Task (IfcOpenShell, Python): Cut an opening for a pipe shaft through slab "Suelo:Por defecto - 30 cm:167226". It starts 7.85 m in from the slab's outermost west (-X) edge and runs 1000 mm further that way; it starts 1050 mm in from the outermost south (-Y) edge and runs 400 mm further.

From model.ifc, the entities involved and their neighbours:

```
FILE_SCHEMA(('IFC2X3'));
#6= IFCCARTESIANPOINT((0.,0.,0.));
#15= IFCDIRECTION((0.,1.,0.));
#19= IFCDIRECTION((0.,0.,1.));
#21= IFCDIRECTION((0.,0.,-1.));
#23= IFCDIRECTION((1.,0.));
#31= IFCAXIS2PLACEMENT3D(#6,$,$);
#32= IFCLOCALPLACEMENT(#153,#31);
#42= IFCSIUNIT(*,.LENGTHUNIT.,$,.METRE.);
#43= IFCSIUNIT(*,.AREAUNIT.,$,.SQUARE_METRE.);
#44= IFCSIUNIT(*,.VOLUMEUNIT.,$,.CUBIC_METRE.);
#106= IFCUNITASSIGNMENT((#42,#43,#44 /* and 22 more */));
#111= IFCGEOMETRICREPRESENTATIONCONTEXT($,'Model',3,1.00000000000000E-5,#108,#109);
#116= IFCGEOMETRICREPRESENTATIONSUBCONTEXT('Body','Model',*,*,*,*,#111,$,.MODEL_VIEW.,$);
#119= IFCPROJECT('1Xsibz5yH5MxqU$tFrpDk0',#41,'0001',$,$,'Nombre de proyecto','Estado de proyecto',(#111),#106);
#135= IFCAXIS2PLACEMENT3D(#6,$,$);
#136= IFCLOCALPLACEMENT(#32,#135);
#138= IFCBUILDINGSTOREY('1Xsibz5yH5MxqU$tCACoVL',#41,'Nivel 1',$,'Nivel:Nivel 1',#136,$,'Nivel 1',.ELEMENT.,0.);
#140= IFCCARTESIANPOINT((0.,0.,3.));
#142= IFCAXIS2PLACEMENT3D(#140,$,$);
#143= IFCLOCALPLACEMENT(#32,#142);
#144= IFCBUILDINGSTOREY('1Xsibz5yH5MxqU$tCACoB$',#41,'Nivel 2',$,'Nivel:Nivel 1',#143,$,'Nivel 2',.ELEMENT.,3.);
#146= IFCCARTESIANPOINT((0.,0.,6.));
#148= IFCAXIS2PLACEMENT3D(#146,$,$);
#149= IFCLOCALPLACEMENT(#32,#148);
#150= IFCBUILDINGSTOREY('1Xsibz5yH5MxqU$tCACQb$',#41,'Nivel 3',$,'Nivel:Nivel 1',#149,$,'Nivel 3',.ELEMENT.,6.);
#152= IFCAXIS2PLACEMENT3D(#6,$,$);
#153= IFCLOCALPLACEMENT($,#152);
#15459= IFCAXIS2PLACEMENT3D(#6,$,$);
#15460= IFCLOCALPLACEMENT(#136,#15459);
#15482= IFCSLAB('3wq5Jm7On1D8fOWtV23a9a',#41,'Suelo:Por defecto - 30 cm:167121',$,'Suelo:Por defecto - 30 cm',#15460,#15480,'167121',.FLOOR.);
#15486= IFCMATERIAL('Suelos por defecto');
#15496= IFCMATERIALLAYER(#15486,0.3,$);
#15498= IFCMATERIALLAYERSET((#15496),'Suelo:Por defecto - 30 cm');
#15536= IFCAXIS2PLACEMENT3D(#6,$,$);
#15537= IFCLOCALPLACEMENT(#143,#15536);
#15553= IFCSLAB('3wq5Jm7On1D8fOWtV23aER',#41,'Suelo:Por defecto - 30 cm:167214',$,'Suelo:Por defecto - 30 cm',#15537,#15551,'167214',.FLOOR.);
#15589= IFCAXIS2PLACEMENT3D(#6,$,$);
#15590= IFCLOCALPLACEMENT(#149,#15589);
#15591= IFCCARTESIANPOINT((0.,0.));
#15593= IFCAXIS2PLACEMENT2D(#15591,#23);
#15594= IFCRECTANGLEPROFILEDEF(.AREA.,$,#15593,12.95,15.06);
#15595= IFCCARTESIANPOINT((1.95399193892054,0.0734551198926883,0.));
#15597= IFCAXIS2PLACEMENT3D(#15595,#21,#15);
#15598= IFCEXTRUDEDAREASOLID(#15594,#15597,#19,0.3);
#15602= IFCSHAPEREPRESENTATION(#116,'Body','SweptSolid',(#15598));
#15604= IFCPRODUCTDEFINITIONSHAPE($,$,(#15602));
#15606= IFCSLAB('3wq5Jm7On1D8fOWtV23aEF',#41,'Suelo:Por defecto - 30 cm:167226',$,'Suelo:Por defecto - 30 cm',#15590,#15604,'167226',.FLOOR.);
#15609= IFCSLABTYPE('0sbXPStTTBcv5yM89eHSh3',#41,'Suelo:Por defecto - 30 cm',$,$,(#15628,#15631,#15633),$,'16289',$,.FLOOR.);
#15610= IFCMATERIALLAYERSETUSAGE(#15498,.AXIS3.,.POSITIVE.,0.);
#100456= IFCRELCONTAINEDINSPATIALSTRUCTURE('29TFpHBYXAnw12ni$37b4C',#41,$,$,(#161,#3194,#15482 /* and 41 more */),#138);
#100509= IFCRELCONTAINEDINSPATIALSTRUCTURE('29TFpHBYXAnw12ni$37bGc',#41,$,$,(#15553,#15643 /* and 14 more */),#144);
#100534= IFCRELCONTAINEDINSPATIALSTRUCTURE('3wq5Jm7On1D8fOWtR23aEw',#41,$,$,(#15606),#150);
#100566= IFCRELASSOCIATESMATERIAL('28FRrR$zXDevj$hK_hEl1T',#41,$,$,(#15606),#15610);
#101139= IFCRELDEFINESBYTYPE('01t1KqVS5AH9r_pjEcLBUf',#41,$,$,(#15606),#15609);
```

```python
import numpy as np
import ifcopenshell
import ifcopenshell.api.feature
import ifcopenshell.api.geometry
import ifcopenshell.api.root
import ifcopenshell.geom
import ifcopenshell.util.placement
import ifcopenshell.util.representation
import ifcopenshell.util.shape
import ifcopenshell.util.unit

model = ifcopenshell.open("model.ifc")
unit_scale = ifcopenshell.util.unit.calculate_unit_scale(model)
settings = ifcopenshell.geom.settings()


def volume(element):
    """Net volume in cubic metres, openings subtracted."""
    shape = ifcopenshell.geom.create_shape(settings, element)
    return ifcopenshell.util.shape.get_volume(shape.geometry)


slab = model.by_guid("3wq5Jm7On1D8fOWtV23aEF")
before = volume(slab)

# Extent in the slab's own axes, in metres. The edges named are its -X and -Y sides.
slab_shape = ifcopenshell.geom.create_shape(settings, slab)
vertices = ifcopenshell.util.shape.get_vertices(slab_shape.geometry)
x_min, y_min, bottom = vertices.min(axis=0)
top = vertices[:, 2].max()

opening = ifcopenshell.api.root.create_entity(model, ifc_class="IfcOpeningElement", name="Pipe shaft opening")
context = ifcopenshell.util.representation.get_context(model, "Model", "Body", "MODEL_VIEW")
width, depth = 1, 0.4
outline = [(0.0, 0.0), (width, 0.0), (width, depth), (0.0, depth), (0.0, 0.0)]
# Overshoot both faces by 50 mm so the cut is clean.
shape = ifcopenshell.api.geometry.add_slab_representation(
    model, context=context, depth=top - bottom + 0.1, polyline=outline
)
ifcopenshell.api.geometry.assign_representation(model, product=opening, representation=shape)

matrix = ifcopenshell.util.placement.get_local_placement(slab.ObjectPlacement)
matrix[:, 3] = matrix @ np.append(np.array([x_min + 7.85, y_min + 1.05, bottom - 0.05]) / unit_scale, 1.0)
ifcopenshell.api.geometry.edit_object_placement(model, product=opening, matrix=matrix, is_si=False)
ifcopenshell.api.feature.add_feature(model, feature=opening, element=slab)

after = volume(slab)

print(f"slab volume {before:.3f} -> {after:.3f} m3")

model.write("model-out.ifc")
```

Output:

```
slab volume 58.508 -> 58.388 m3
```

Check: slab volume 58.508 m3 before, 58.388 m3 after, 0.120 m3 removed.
